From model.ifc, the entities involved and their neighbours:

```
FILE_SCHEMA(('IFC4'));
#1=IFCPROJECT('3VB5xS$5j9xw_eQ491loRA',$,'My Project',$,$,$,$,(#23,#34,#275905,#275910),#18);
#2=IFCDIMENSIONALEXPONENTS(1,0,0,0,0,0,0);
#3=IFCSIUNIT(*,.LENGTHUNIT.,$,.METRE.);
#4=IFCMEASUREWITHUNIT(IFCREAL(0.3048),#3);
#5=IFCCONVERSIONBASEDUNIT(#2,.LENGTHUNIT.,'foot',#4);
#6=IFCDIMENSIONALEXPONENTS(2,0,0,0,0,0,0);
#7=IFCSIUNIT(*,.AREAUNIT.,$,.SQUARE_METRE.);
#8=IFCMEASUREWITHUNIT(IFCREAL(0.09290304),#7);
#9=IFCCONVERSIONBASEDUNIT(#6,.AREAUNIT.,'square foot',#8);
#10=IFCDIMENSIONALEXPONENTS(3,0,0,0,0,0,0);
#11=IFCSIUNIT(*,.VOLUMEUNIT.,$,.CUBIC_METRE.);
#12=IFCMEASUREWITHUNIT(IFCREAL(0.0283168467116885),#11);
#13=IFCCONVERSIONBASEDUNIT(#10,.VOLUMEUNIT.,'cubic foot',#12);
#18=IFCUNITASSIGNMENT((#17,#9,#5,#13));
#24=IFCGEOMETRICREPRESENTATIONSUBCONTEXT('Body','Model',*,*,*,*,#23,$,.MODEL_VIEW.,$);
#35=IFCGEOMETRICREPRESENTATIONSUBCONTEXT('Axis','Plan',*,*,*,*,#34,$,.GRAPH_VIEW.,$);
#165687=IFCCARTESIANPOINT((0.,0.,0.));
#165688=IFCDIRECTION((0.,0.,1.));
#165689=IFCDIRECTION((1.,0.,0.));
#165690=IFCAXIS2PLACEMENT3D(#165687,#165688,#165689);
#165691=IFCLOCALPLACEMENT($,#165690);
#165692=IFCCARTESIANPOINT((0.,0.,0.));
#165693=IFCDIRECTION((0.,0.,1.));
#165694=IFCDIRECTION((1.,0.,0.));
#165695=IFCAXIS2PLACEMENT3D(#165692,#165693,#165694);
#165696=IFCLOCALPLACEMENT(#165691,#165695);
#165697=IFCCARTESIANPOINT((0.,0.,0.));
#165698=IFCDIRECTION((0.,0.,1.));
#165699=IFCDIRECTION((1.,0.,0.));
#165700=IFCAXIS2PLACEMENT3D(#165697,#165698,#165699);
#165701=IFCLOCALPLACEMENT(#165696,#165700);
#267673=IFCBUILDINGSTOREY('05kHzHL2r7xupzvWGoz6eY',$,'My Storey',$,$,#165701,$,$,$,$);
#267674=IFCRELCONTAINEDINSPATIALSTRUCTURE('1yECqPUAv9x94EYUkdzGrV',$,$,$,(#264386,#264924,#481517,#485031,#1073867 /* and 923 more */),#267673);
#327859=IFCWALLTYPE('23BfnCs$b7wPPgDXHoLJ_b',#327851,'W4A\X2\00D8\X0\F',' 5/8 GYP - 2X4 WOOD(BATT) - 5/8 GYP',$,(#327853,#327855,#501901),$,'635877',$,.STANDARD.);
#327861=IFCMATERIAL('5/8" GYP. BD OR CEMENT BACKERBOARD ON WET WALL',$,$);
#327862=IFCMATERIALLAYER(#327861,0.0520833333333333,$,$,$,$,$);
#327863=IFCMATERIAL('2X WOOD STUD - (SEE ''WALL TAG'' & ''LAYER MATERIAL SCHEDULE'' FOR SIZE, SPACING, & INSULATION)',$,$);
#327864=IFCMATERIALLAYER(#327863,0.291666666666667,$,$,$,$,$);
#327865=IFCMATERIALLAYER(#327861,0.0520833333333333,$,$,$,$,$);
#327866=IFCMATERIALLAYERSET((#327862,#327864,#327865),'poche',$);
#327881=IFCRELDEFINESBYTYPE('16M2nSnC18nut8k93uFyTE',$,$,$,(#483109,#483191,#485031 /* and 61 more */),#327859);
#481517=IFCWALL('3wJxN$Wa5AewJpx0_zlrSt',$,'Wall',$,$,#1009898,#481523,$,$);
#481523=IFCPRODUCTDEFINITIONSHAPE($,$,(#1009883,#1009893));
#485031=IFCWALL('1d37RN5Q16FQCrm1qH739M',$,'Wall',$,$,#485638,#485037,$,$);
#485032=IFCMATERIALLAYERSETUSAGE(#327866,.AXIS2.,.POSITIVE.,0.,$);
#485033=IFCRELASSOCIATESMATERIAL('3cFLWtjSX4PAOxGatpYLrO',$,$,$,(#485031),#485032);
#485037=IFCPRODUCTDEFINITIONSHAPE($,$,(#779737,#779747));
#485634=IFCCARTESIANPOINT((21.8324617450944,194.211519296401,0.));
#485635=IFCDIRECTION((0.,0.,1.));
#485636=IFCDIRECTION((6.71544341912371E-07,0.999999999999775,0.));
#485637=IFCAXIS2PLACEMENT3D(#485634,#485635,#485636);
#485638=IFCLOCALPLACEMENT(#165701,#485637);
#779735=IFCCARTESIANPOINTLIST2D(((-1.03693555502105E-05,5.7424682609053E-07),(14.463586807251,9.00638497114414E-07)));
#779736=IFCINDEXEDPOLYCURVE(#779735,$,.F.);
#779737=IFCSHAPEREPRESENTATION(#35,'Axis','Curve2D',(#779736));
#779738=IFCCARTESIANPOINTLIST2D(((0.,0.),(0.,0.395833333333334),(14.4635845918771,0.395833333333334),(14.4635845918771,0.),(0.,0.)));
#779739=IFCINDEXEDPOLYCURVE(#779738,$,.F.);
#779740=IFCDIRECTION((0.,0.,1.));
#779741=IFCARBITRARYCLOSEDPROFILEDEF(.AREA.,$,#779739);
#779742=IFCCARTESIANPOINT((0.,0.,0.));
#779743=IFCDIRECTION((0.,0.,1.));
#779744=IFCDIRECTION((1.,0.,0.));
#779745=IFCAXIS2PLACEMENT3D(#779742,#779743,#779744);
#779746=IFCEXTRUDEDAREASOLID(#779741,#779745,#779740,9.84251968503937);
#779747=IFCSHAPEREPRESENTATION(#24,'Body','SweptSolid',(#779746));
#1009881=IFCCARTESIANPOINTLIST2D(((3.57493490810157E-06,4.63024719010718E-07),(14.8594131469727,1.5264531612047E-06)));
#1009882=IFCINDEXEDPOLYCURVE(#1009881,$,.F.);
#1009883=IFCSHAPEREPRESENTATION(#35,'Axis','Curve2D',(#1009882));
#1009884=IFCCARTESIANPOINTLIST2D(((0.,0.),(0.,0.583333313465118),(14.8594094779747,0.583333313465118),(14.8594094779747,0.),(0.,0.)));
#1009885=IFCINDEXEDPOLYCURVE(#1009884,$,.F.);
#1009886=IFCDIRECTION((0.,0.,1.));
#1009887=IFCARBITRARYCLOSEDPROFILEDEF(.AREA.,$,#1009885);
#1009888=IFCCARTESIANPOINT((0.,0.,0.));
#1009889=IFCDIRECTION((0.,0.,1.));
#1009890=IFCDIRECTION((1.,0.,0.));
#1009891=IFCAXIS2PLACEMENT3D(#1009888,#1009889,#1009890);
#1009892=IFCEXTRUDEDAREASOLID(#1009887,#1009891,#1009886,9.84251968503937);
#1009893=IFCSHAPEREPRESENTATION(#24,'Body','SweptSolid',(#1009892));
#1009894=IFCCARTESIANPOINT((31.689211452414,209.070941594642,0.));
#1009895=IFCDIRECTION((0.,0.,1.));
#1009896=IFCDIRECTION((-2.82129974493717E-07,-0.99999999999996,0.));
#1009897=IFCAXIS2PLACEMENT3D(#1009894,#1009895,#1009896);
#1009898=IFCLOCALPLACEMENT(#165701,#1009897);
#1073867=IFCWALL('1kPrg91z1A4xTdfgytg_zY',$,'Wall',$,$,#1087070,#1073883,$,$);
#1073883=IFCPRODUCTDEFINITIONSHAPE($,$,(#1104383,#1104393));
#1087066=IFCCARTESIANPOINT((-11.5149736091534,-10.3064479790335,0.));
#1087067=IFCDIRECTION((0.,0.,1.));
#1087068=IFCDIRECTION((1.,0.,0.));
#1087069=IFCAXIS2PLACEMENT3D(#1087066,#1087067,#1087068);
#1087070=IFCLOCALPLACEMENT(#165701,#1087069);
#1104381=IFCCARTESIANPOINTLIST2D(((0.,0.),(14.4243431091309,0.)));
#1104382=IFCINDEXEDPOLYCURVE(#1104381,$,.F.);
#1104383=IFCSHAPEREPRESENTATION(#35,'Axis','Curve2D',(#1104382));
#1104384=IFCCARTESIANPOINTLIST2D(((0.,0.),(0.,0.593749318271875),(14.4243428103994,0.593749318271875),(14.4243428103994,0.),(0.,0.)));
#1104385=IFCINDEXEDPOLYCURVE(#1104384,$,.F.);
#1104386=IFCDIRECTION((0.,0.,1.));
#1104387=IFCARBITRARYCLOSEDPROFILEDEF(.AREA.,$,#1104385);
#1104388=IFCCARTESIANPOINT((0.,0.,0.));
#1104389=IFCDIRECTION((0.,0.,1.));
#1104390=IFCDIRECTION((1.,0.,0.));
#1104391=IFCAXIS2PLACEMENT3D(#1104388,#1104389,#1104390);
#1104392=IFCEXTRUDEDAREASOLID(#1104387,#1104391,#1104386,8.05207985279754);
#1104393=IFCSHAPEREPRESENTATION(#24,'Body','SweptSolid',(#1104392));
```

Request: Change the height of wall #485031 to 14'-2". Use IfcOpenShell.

```python
import ifcopenshell
import ifcopenshell.geom
import ifcopenshell.util.representation
import ifcopenshell.util.shape
import ifcopenshell.util.unit

model = ifcopenshell.open("model.ifc")
unit_scale = ifcopenshell.util.unit.calculate_unit_scale(model)
settings = ifcopenshell.geom.settings()


def volume(element):
    """Net volume in cubic metres, openings subtracted."""
    shape = ifcopenshell.geom.create_shape(settings, element)
    return ifcopenshell.util.shape.get_volume(shape.geometry)


wall = model.by_id(485031)
before = volume(wall)

body = ifcopenshell.util.representation.get_representation(wall, "Model", "Body")
solid = body.Items[0]
old_height = solid.Depth
solid.Depth = 170 * 0.0254 / unit_scale
after = volume(wall)

print(f"height {old_height:g} -> {solid.Depth:g}, volume {before:.3f} -> {after:.3f} m3")

model.write("model_v2.ifc")
```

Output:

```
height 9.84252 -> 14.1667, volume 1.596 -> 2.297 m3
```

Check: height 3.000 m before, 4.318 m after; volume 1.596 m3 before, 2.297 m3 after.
